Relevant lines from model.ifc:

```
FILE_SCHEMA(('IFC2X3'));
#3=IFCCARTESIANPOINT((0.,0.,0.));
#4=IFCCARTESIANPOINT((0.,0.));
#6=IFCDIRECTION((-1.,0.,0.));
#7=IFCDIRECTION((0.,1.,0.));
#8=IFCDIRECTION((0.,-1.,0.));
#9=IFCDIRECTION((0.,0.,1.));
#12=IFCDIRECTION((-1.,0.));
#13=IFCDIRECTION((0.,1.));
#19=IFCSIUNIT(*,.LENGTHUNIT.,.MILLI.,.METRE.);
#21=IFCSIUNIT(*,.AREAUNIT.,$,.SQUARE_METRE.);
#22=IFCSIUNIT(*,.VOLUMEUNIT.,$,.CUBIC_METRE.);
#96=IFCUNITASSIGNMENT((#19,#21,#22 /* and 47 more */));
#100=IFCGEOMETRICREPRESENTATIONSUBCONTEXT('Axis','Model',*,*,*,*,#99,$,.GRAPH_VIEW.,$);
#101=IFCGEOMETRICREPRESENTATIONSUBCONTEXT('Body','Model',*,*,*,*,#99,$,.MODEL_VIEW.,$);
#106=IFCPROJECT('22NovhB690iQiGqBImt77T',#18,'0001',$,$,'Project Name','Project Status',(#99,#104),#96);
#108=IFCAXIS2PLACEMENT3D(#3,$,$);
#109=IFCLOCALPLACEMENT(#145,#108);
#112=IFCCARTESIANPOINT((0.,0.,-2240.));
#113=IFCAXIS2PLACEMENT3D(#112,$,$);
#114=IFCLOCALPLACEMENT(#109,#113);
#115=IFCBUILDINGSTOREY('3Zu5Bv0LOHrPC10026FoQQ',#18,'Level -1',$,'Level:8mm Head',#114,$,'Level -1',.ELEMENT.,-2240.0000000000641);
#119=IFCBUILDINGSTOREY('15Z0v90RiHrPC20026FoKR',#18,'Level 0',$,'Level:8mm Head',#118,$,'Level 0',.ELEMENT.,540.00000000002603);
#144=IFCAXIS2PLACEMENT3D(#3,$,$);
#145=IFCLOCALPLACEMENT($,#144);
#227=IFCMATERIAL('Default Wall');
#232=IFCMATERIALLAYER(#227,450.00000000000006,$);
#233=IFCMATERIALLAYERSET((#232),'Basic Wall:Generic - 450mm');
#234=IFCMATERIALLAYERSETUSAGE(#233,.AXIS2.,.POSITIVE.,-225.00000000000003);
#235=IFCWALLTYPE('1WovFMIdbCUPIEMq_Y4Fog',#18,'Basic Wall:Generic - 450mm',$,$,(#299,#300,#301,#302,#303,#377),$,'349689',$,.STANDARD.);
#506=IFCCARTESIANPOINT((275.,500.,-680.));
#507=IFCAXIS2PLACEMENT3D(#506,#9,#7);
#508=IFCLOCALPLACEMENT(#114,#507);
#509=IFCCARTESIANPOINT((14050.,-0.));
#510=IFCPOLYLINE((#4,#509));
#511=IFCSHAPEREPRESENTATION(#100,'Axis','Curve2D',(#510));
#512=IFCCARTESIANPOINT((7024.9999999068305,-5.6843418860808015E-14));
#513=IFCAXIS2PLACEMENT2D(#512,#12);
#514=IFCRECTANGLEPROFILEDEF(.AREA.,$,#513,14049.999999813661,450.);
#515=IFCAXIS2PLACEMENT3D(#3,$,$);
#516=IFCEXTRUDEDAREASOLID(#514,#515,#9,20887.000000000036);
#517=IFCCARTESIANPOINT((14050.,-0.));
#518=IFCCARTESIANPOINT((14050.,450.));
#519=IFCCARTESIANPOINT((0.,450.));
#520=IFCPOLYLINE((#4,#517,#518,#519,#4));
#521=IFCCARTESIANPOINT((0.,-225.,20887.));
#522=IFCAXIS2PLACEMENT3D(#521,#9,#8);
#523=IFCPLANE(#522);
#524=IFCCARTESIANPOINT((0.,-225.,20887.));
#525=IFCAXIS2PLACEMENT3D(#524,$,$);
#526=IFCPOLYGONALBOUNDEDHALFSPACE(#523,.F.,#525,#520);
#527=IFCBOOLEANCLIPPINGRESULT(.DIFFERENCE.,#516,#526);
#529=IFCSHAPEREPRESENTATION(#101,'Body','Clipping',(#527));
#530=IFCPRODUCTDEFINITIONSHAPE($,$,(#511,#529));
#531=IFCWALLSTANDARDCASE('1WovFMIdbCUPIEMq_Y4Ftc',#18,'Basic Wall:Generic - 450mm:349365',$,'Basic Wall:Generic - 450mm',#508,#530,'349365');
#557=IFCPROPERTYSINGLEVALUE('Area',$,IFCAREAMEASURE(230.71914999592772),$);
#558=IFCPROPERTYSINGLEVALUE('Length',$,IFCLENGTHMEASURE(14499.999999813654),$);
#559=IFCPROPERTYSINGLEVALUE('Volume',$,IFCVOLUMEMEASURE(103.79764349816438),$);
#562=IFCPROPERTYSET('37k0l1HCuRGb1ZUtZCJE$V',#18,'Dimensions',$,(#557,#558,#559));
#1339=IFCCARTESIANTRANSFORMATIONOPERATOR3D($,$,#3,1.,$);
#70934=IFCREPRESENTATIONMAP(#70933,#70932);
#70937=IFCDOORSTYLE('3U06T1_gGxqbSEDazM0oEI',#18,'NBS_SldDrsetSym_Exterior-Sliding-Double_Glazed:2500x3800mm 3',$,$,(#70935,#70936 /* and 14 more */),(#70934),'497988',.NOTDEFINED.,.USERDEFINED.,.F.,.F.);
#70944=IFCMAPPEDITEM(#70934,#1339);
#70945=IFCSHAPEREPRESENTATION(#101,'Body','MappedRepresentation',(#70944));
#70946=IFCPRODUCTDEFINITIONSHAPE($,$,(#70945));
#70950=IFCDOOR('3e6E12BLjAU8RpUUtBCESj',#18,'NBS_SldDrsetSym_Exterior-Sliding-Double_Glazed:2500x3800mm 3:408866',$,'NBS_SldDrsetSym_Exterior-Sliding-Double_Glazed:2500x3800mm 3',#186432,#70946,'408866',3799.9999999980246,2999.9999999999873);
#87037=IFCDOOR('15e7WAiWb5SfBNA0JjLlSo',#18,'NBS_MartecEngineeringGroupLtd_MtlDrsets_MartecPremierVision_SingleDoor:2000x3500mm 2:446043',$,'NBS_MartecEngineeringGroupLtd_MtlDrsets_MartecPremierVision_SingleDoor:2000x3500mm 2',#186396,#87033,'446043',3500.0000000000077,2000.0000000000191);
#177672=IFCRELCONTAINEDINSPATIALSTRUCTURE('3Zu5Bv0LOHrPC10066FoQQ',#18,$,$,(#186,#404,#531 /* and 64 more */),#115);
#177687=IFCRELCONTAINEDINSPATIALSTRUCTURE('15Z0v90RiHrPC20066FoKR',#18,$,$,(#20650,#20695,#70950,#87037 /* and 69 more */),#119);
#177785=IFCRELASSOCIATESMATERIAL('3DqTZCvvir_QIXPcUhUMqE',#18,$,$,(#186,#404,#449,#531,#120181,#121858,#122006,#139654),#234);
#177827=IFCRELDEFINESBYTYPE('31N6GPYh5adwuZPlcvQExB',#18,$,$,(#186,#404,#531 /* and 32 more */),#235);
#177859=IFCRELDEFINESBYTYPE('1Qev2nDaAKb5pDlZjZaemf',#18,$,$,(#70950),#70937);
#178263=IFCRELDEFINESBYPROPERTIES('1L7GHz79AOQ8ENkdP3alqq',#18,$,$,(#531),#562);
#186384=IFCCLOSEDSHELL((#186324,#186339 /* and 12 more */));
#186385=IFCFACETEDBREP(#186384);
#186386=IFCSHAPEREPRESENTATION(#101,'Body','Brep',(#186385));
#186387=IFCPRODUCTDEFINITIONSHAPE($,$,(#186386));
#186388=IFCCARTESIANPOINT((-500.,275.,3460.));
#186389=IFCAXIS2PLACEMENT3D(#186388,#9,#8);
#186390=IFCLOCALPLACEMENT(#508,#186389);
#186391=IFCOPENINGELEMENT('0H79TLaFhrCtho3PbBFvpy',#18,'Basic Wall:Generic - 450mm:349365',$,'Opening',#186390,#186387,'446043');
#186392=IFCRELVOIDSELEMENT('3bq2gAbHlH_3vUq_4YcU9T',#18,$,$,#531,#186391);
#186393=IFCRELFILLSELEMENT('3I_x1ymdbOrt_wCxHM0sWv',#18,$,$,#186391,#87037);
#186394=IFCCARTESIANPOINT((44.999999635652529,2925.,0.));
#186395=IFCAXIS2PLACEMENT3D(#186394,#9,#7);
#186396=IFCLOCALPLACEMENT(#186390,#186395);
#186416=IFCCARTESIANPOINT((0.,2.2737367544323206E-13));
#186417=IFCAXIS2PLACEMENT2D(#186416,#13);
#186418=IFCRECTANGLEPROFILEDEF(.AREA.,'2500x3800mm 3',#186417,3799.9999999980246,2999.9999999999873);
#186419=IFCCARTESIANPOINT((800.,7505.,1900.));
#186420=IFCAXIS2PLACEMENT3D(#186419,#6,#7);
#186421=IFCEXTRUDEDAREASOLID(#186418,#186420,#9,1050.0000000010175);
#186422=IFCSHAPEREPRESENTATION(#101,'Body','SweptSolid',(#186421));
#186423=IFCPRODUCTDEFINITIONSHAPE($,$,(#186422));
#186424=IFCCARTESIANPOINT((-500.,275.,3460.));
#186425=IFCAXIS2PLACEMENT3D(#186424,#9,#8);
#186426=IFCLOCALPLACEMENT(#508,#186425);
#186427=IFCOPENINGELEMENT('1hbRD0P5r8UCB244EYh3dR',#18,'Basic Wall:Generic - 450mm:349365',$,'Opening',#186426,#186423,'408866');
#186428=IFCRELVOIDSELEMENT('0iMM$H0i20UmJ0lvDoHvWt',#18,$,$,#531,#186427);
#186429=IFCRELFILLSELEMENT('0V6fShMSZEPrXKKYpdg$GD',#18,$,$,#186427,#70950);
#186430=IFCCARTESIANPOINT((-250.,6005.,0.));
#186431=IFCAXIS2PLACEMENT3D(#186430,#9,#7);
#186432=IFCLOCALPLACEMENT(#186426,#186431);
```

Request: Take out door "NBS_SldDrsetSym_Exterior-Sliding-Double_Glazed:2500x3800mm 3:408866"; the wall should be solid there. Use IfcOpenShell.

```python
import ifcopenshell
import ifcopenshell.api.feature
import ifcopenshell.api.pset
import ifcopenshell.api.root
import ifcopenshell.geom
import ifcopenshell.util.element
import ifcopenshell.util.shape
import ifcopenshell.util.unit

model = ifcopenshell.open("model.ifc")
area_scale = ifcopenshell.util.unit.calculate_unit_scale(model, "AREAUNIT")
volume_scale = ifcopenshell.util.unit.calculate_unit_scale(model, "VOLUMEUNIT")
settings = ifcopenshell.geom.settings()


def volume(element):
    """Net volume in cubic metres, openings subtracted."""
    shape = ifcopenshell.geom.create_shape(settings, element)
    return ifcopenshell.util.shape.get_volume(shape.geometry)


door = model.by_guid("3e6E12BLjAU8RpUUtBCESj")
opening = door.FillsVoids[0].RelatingOpeningElement
wall = opening.VoidsElements[0].RelatingBuildingElement
before = volume(wall)

ifcopenshell.api.root.remove_product(model, product=door)
ifcopenshell.api.feature.remove_feature(model, feature=opening)

after = volume(wall)
thickness = 0.45  # wall thickness in metres

# Update the wall's stored quantities.
pset = model.by_id(ifcopenshell.util.element.get_pset(wall, "Dimensions", should_inherit=False)["id"])
ifcopenshell.api.pset.edit_pset(model, pset=pset, properties={
    "Area": model.create_entity("IfcAreaMeasure", after / thickness / area_scale),
    "Volume": model.create_entity("IfcVolumeMeasure", after / volume_scale),
})

print(f"wall volume {before:.3f} -> {after:.3f} m3")

model.write("model_updated.ifc")
```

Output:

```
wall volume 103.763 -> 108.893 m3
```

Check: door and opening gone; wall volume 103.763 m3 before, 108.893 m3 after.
